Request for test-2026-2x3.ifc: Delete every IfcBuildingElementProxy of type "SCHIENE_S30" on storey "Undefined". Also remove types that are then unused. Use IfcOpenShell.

First a look at what the model holds.

```python
import ifcopenshell
import ifcopenshell.util.element

model = ifcopenshell.open("test-2026-2x3.ifc")
print(model.schema)
storey = next(s for s in model.by_type("IfcBuildingStorey") if s.Name == "Undefined")
proxies = [e for e in ifcopenshell.util.element.get_decomposition(storey) if e.is_a("IfcBuildingElementProxy")]
seen = {}
for e in proxies:
    element_type = ifcopenshell.util.element.get_type(e)
    name = element_type.Name if element_type not in (None, e) else None
    seen[name] = seen.get(name, 0) + 1
for name, count in sorted(seen.items(), key=str):
    print(count, "x", name)
```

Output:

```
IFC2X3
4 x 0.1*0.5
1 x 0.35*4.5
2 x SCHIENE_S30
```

```python
import ifcopenshell
import ifcopenshell.api.root
import ifcopenshell.util.element

model = ifcopenshell.open("test-2026-2x3.ifc")

storey = next(s for s in model.by_type("IfcBuildingStorey") if s.Name == "Undefined")
proxies = [e for e in ifcopenshell.util.element.get_decomposition(storey) if e.is_a("IfcBuildingElementProxy")]
targets = [e for e in proxies if (t := ifcopenshell.util.element.get_type(e)) not in (None, e) and t.Name == "SCHIENE_S30"]
types = {ifcopenshell.util.element.get_type(e) for e in targets} - {None, *targets}

for e in targets:
    ifcopenshell.api.root.remove_product(model, product=e)
print(len(targets), "removed")

unused = [t for t in types if not ifcopenshell.util.element.get_types(t)]
for t in unused:
    ifcopenshell.api.root.remove_product(model, product=t)
print(len(unused), "unused types removed")

model.write("test-2026-2x3_updated.ifc")
```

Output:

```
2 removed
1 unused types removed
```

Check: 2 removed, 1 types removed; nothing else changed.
